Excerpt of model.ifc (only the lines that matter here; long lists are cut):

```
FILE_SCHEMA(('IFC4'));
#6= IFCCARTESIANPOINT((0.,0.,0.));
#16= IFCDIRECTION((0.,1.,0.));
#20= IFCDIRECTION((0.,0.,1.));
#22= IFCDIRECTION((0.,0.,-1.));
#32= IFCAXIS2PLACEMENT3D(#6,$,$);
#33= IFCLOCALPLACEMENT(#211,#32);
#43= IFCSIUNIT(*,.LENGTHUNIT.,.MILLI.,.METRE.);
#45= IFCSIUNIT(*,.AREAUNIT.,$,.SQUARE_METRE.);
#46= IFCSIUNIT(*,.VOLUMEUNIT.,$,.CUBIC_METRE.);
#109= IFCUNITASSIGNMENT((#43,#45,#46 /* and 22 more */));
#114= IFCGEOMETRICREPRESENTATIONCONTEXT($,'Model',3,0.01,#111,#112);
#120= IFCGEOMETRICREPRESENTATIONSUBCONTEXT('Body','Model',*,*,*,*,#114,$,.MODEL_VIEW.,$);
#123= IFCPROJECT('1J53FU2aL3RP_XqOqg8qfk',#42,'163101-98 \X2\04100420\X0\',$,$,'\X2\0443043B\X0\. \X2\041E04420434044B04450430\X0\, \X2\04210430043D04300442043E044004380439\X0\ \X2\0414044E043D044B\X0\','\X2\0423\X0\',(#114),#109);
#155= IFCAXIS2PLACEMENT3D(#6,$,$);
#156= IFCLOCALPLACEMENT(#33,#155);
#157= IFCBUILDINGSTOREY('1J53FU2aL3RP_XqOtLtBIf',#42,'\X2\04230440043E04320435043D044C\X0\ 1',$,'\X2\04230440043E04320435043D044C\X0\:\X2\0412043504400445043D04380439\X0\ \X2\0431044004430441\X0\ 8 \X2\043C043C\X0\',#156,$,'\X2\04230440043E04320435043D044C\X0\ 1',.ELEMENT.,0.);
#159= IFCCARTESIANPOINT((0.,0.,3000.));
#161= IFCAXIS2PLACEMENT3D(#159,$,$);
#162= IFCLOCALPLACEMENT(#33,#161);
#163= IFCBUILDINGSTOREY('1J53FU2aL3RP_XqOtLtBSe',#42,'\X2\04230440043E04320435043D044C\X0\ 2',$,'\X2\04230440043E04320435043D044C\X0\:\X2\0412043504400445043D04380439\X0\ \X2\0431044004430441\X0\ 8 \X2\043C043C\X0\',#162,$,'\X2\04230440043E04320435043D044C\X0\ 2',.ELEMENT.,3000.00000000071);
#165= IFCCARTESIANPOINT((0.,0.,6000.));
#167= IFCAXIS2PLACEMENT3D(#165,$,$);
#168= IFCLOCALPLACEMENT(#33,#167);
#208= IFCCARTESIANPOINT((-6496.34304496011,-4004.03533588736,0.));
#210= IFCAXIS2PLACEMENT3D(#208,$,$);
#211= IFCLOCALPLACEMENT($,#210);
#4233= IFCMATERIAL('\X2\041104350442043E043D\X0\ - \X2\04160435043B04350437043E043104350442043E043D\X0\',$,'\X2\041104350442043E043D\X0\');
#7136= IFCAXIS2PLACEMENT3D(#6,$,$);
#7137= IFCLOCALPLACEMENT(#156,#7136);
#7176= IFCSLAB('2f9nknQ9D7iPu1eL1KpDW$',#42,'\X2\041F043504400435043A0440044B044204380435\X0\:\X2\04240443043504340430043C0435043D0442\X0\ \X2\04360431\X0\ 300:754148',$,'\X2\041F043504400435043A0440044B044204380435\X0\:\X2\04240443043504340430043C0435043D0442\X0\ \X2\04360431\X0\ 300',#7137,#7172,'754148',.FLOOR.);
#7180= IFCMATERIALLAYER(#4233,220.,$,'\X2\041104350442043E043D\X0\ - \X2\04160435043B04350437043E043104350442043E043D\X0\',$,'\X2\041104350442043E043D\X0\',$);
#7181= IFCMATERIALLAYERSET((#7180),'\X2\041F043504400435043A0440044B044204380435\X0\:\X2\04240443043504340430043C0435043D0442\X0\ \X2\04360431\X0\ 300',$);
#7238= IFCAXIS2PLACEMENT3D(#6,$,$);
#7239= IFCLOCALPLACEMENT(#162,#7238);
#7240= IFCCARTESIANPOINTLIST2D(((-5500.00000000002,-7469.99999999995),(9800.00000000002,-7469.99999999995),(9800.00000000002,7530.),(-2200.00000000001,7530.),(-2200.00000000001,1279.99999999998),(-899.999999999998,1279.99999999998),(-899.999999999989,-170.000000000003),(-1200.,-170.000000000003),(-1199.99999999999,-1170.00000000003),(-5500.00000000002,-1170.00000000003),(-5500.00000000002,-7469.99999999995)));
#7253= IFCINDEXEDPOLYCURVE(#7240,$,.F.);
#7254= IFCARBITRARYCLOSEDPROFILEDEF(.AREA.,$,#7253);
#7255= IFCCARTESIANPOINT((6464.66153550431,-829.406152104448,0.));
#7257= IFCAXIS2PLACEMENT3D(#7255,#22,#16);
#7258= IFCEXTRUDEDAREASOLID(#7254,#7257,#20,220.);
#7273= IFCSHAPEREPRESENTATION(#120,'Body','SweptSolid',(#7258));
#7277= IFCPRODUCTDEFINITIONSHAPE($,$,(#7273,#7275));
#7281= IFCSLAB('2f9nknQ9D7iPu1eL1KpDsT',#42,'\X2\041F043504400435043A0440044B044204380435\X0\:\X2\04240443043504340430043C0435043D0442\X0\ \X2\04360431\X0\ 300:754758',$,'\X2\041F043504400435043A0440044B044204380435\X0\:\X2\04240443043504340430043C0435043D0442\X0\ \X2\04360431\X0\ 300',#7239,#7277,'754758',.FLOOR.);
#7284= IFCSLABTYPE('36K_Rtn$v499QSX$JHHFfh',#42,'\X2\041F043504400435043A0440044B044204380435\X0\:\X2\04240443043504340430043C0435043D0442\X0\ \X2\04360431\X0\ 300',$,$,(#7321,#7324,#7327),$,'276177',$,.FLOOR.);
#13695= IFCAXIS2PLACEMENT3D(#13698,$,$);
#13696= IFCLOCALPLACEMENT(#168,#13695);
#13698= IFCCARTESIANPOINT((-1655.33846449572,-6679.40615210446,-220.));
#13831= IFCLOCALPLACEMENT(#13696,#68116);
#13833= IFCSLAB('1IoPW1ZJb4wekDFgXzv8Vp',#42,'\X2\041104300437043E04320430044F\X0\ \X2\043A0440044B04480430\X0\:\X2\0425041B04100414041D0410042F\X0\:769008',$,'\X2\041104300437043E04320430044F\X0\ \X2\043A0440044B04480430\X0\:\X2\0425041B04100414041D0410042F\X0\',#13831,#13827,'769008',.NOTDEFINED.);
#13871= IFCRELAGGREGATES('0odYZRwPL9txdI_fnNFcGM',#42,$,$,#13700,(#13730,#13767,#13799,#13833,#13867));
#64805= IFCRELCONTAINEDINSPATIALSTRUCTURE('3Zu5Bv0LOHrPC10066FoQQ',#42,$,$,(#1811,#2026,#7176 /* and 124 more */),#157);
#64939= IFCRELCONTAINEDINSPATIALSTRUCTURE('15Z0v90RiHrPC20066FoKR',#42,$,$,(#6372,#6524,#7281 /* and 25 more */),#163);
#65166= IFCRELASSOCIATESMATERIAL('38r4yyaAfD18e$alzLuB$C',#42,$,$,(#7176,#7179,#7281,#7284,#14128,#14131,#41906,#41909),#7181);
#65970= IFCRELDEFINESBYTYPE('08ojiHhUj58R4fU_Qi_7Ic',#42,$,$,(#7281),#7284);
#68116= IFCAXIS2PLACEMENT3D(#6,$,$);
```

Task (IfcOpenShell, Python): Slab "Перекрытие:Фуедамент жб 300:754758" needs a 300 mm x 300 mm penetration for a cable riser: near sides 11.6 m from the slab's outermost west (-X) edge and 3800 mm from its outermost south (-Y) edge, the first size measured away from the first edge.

```python
import numpy as np
import ifcopenshell
import ifcopenshell.api.feature
import ifcopenshell.api.geometry
import ifcopenshell.api.root
import ifcopenshell.geom
import ifcopenshell.util.placement
import ifcopenshell.util.representation
import ifcopenshell.util.shape
import ifcopenshell.util.unit

model = ifcopenshell.open("model.ifc")
unit_scale = ifcopenshell.util.unit.calculate_unit_scale(model)
settings = ifcopenshell.geom.settings()


def volume(element):
    """Net volume in cubic metres, openings subtracted."""
    shape = ifcopenshell.geom.create_shape(settings, element)
    return ifcopenshell.util.shape.get_volume(shape.geometry)


slab = model.by_id(7281)
before = volume(slab)

# Extent in the slab's own axes, in metres. The edges named are its -X and -Y sides.
slab_shape = ifcopenshell.geom.create_shape(settings, slab)
vertices = ifcopenshell.util.shape.get_vertices(slab_shape.geometry)
x_min, y_min, bottom = vertices.min(axis=0)
top = vertices[:, 2].max()

opening = ifcopenshell.api.root.create_entity(model, ifc_class="IfcOpeningElement", name="Cable riser opening", predefined_type="OPENING")
context = ifcopenshell.util.representation.get_context(model, "Model", "Body", "MODEL_VIEW")
width, depth = 0.3, 0.3
outline = [(0.0, 0.0), (width, 0.0), (width, depth), (0.0, depth), (0.0, 0.0)]
# Overshoot both faces by 50 mm so the cut is clean.
shape = ifcopenshell.api.geometry.add_slab_representation(
    model, context=context, depth=top - bottom + 0.1, polyline=outline
)
ifcopenshell.api.geometry.assign_representation(model, product=opening, representation=shape)

matrix = ifcopenshell.util.placement.get_local_placement(slab.ObjectPlacement)
matrix[:, 3] = matrix @ np.append(np.array([x_min + 11.6, y_min + 3.8, bottom - 0.05]) / unit_scale, 1.0)
ifcopenshell.api.geometry.edit_object_placement(model, product=opening, matrix=matrix, is_si=False)
ifcopenshell.api.feature.add_feature(model, feature=opening, element=slab)

after = volume(slab)

print(f"slab volume {before:.3f} -> {after:.3f} m3")

model.write("model_v2.ifc")
```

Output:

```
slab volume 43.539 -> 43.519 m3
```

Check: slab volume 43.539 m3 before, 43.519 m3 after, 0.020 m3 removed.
